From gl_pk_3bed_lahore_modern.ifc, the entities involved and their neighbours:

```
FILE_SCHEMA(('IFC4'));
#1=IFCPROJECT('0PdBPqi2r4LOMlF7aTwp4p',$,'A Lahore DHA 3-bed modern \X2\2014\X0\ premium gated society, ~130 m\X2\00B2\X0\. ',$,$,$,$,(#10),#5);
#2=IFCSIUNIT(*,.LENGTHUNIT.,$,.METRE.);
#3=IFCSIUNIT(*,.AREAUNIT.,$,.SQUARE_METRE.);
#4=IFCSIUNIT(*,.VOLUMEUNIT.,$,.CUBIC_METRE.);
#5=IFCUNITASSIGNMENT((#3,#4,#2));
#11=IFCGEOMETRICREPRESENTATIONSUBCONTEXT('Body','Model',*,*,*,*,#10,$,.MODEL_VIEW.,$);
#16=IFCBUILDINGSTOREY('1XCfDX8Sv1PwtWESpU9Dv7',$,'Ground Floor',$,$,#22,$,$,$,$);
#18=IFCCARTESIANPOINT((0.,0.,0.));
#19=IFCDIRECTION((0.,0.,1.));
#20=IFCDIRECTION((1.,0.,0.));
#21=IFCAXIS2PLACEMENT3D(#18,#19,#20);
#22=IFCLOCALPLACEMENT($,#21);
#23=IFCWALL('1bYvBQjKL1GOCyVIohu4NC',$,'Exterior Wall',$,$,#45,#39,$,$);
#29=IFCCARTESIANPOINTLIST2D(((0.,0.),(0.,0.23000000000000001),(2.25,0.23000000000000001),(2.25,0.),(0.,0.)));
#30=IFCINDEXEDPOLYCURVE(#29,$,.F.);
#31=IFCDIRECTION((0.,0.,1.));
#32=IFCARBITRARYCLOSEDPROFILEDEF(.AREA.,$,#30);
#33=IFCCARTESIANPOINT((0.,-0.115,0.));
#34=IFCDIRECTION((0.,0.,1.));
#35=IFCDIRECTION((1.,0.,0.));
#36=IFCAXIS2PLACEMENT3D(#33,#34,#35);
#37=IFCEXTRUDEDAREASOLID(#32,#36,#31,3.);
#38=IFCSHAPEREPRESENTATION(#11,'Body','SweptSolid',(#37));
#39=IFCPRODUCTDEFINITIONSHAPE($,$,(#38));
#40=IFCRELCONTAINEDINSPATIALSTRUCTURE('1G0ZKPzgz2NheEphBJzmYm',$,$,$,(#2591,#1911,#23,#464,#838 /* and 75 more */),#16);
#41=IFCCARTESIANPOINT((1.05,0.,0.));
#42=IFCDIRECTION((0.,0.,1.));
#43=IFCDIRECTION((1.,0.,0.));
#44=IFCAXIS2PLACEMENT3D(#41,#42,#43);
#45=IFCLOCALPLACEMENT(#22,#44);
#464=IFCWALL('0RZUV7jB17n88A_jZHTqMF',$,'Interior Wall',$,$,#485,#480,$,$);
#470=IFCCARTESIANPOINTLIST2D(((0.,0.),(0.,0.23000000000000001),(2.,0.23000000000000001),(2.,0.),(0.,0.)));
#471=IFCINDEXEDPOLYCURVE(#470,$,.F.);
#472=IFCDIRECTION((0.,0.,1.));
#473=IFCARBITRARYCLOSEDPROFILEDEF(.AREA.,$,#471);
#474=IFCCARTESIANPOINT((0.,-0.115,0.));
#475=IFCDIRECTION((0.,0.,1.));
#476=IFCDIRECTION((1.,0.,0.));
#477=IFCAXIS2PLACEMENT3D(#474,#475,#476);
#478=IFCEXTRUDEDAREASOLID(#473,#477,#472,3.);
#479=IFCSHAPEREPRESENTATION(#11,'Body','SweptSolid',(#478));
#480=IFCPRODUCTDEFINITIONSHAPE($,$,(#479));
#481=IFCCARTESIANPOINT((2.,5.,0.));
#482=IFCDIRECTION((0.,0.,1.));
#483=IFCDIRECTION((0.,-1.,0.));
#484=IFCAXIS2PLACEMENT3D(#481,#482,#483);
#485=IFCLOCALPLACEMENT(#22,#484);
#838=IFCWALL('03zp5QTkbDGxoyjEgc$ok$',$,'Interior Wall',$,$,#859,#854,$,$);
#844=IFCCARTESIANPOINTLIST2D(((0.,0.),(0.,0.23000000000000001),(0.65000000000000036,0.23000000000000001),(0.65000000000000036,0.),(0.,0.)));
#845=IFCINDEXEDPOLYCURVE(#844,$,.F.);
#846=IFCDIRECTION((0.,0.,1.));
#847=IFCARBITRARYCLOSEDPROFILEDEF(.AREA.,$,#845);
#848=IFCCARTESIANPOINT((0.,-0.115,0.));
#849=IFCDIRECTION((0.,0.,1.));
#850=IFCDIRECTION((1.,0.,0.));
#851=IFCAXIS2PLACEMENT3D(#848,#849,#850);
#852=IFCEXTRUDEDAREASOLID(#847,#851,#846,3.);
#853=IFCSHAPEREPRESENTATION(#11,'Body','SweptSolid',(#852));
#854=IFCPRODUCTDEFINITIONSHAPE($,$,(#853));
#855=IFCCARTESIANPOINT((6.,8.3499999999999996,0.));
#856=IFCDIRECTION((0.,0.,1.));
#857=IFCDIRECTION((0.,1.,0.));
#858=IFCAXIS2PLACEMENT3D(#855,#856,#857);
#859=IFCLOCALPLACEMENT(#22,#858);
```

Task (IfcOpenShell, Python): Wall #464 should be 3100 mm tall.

```python
import ifcopenshell
import ifcopenshell.geom
import ifcopenshell.util.representation
import ifcopenshell.util.shape
import ifcopenshell.util.unit

model = ifcopenshell.open("gl_pk_3bed_lahore_modern.ifc")
unit_scale = ifcopenshell.util.unit.calculate_unit_scale(model)
settings = ifcopenshell.geom.settings()


def volume(element):
    """Net volume in cubic metres, openings subtracted."""
    shape = ifcopenshell.geom.create_shape(settings, element)
    return ifcopenshell.util.shape.get_volume(shape.geometry)


wall = model.by_guid("0RZUV7jB17n88A_jZHTqMF")
before = volume(wall)

body = ifcopenshell.util.representation.get_representation(wall, "Model", "Body")
solid = body.Items[0]
old_height = solid.Depth
solid.Depth = 3.1 / unit_scale
after = volume(wall)

print(f"height {old_height:g} -> {solid.Depth:g}, volume {before:.3f} -> {after:.3f} m3")

model.write("gl_pk_3bed_lahore_modern-out.ifc")
```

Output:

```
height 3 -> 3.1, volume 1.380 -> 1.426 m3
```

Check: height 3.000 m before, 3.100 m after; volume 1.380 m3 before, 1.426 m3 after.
